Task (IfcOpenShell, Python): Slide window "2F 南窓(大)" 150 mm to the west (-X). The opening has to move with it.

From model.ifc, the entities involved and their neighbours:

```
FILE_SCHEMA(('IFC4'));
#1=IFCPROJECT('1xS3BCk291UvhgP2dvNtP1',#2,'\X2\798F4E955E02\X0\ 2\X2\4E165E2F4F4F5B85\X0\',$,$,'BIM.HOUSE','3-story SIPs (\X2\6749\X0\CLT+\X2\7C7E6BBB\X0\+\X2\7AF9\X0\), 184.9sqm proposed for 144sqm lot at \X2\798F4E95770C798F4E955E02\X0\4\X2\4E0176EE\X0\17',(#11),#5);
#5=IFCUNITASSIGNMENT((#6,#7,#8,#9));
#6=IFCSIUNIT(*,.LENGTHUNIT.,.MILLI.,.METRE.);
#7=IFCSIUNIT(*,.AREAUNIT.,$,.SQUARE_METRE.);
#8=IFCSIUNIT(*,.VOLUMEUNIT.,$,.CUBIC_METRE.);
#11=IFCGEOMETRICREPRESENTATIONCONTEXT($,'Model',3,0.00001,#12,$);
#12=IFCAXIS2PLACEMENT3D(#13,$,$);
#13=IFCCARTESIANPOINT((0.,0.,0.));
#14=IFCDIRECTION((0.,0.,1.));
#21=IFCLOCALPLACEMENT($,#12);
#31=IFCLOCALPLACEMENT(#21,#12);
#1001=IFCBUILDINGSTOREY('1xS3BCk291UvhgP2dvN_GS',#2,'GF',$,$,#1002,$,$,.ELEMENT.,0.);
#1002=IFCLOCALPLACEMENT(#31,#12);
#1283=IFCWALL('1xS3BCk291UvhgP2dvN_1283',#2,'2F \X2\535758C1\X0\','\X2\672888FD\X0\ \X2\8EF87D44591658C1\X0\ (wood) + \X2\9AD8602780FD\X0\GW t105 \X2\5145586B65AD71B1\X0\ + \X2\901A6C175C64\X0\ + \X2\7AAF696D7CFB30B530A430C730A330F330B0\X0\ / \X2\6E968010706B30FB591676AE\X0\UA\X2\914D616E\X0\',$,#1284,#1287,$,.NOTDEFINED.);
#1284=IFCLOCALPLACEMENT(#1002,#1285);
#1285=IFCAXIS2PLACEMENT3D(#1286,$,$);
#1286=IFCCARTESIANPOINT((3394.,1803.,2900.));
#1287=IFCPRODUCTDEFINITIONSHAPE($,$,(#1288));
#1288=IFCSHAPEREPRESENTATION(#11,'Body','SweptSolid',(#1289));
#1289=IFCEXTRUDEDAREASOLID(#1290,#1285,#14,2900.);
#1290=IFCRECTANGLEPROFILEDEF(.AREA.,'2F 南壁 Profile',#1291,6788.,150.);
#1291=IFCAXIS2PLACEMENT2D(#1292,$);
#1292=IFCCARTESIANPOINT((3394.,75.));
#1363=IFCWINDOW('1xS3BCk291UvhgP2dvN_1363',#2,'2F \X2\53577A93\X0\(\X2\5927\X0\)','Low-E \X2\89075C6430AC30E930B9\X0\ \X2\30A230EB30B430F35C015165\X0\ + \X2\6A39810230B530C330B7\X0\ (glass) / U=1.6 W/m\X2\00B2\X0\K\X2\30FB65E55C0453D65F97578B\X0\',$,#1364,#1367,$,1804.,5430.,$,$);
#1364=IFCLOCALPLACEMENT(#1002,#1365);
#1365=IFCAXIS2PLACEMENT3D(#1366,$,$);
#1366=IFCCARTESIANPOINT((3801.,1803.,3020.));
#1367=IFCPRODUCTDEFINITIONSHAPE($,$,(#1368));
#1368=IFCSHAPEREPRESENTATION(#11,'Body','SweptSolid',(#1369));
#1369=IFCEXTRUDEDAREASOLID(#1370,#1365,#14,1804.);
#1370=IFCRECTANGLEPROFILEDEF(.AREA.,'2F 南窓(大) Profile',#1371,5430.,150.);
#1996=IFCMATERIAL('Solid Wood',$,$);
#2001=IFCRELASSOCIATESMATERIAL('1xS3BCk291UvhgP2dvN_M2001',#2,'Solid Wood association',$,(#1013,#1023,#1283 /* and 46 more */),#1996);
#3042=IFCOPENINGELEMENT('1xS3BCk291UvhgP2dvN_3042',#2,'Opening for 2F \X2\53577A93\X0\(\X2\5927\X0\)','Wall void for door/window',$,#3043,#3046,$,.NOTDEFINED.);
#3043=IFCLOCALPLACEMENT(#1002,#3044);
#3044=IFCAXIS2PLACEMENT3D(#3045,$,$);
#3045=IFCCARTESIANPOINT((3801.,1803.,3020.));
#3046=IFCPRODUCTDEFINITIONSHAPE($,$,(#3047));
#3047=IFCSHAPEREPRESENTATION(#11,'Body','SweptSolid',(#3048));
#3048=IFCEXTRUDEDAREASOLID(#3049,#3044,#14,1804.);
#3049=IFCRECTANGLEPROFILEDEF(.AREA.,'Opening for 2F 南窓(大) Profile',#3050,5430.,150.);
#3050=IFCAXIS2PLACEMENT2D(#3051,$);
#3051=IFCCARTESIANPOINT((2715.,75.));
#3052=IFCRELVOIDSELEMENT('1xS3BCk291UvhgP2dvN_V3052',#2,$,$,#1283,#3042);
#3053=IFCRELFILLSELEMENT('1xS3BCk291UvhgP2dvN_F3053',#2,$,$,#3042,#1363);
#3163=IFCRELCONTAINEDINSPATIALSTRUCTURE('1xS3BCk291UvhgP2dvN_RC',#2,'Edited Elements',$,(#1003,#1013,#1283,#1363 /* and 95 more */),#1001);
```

```python
import ifcopenshell
import ifcopenshell.api.geometry
import ifcopenshell.util.placement
import ifcopenshell.util.unit

model = ifcopenshell.open("model.ifc")
unit_scale = ifcopenshell.util.unit.calculate_unit_scale(model)

window = model.by_guid("1xS3BCk291UvhgP2dvN_1363")
opening = window.FillsVoids[0].RelatingOpeningElement
wall = opening.VoidsElements[0].RelatingBuildingElement

wall_matrix = ifcopenshell.util.placement.get_local_placement(wall.ObjectPlacement)
shift = wall_matrix[:3, 0] * -0.15 / unit_scale
before = ifcopenshell.util.placement.get_local_placement(window.ObjectPlacement)[:3, 3].copy()

# The window is not placed relative to its opening, so move both.
for product in (opening, window):
    matrix = ifcopenshell.util.placement.get_local_placement(product.ObjectPlacement)
    matrix[:3, 3] += shift
    ifcopenshell.api.geometry.edit_object_placement(model, product=product, matrix=matrix, is_si=False)

after = ifcopenshell.util.placement.get_local_placement(window.ObjectPlacement)[:3, 3]
print("window moved by", (after - before).round(3) + 0.0)

model.write("model_updated.ifc")
```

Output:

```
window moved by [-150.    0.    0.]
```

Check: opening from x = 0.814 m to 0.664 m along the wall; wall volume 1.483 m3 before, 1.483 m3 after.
